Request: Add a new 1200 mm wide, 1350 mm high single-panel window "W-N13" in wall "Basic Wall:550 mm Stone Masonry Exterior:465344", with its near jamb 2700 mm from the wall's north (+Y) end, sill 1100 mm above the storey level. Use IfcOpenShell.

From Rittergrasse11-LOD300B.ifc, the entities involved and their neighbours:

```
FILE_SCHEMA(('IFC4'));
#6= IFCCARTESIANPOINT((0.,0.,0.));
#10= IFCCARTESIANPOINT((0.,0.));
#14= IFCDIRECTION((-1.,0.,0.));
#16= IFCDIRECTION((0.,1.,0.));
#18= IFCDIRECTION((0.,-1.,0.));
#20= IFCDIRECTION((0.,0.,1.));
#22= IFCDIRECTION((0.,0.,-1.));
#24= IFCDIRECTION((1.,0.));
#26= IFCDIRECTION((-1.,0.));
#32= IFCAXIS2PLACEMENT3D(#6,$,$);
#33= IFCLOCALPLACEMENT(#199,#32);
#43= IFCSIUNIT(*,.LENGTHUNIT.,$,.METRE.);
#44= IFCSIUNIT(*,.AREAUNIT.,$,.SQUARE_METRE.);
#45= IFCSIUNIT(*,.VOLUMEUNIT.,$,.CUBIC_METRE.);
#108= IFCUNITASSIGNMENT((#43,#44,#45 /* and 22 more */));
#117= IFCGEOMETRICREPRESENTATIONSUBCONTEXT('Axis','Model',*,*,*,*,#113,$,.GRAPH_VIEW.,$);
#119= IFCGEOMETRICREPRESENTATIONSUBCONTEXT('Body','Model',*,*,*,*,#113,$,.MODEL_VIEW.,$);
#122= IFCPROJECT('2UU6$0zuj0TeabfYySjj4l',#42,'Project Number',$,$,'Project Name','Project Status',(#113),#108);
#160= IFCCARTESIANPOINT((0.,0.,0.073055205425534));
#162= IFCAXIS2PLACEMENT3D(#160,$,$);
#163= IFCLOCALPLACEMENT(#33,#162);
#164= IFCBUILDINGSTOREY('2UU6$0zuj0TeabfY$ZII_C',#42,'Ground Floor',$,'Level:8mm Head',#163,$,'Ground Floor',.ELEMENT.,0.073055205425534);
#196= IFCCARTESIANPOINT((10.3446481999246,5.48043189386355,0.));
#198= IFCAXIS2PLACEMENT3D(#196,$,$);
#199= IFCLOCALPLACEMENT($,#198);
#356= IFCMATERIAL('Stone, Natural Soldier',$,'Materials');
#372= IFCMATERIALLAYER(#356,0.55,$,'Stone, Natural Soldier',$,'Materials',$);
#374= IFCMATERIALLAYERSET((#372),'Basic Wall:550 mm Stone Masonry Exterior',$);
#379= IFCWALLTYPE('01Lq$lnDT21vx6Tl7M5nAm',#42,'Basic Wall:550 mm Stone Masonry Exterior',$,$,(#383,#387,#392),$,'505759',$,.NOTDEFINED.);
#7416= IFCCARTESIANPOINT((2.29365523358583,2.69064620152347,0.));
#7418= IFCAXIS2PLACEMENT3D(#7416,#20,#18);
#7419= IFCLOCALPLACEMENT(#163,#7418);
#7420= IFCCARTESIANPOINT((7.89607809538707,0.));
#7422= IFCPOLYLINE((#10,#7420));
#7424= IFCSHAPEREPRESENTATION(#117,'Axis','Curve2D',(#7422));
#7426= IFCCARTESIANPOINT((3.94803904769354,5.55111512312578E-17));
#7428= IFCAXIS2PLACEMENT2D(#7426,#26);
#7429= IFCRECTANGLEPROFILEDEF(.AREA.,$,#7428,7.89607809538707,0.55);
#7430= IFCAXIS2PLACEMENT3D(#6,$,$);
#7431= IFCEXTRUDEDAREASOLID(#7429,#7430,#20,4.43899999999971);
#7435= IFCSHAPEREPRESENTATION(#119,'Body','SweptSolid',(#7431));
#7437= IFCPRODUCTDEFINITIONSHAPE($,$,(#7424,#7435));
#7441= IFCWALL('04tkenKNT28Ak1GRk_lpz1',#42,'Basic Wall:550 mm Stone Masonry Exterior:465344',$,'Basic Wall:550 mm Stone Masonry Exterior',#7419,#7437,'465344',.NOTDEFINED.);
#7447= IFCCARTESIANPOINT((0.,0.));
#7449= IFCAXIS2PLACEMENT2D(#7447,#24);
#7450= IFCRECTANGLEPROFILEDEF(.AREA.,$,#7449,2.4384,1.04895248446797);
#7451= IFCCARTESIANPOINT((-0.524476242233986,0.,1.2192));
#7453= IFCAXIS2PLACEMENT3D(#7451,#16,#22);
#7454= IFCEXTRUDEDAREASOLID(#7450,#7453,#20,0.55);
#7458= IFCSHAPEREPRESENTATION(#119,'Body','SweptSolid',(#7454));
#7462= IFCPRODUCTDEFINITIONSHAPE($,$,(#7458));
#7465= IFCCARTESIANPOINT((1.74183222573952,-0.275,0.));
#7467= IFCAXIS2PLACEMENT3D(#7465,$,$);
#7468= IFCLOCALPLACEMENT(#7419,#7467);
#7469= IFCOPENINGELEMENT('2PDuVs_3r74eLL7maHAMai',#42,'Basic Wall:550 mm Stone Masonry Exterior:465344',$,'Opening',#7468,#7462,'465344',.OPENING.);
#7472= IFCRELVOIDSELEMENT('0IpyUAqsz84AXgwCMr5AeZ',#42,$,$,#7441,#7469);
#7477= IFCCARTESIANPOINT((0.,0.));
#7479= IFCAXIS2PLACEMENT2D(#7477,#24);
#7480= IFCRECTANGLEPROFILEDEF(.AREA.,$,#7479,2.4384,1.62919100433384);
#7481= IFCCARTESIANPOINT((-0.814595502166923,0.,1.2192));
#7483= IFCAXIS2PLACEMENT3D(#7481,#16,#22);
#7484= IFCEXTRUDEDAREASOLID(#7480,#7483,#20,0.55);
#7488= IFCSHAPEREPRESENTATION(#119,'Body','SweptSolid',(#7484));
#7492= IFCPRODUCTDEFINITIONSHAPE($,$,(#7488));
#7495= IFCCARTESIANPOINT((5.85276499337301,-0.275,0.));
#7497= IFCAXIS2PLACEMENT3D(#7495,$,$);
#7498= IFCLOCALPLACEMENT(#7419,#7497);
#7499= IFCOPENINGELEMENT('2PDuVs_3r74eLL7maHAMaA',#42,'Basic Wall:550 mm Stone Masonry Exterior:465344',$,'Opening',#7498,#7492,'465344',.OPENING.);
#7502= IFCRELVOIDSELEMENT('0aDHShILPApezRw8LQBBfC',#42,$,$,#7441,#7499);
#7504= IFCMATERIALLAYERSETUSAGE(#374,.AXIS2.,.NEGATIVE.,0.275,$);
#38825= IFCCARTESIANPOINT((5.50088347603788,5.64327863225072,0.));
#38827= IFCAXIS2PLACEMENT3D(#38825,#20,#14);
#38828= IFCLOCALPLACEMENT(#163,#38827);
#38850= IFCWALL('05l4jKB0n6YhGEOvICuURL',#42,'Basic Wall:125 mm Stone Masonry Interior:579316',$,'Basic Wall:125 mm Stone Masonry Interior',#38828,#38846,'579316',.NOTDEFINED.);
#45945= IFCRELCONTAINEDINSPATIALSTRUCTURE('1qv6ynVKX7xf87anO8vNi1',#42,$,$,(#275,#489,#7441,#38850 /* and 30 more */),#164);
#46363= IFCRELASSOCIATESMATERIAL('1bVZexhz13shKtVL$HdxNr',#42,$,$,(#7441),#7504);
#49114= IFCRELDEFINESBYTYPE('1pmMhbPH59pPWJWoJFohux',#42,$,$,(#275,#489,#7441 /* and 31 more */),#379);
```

```python
import numpy as np
import ifcopenshell
import ifcopenshell.api.feature
import ifcopenshell.api.geometry
import ifcopenshell.api.root
import ifcopenshell.api.spatial
import ifcopenshell.geom
import ifcopenshell.util.element
import ifcopenshell.util.placement
import ifcopenshell.util.representation
import ifcopenshell.util.shape
import ifcopenshell.util.unit

model = ifcopenshell.open("Rittergrasse11-LOD300B.ifc")
unit_scale = ifcopenshell.util.unit.calculate_unit_scale(model)
settings = ifcopenshell.geom.settings()


def volume(element):
    """Net volume in cubic metres, openings subtracted."""
    shape = ifcopenshell.geom.create_shape(settings, element)
    return ifcopenshell.util.shape.get_volume(shape.geometry)


wall = model.by_guid("04tkenKNT28Ak1GRk_lpz1")
storey = ifcopenshell.util.element.get_container(wall, ifc_class="IfcBuildingStorey")
context = ifcopenshell.util.representation.get_context(model, "Model", "Body", "MODEL_VIEW")
before = volume(wall)

width, height, from_end, sill = 1.2, 1.35, 2.7, 1.1  # metres

# The wall runs along its own X axis, and the end named is its -X end.
wall_shape = ifcopenshell.geom.create_shape(settings, wall)
x, y, z = ifcopenshell.util.shape.get_vertices(wall_shape.geometry).T
start = x.min() + from_end
face, thickness = float(y.min()), float(y.max() - y.min())
wall_matrix = ifcopenshell.util.placement.get_local_placement(wall.ObjectPlacement)
level = ifcopenshell.util.placement.get_local_placement(storey.ObjectPlacement)[2, 3]


def in_wall(x, y):
    """Placement at x, y metres in the wall's axes, at sill height."""
    matrix = wall_matrix.copy()
    matrix[:, 3] = wall_matrix @ np.array([x / unit_scale, y / unit_scale, 0.0, 1.0])
    matrix[2, 3] = level + sill / unit_scale
    return matrix


# Opening: a box that overshoots both wall faces by 50 mm.
opening = ifcopenshell.api.root.create_entity(model, ifc_class="IfcOpeningElement", predefined_type="OPENING")
box = ifcopenshell.api.geometry.add_wall_representation(
    model, context=context, length=width, height=height, thickness=thickness + 0.1
)
ifcopenshell.api.geometry.assign_representation(model, product=opening, representation=box)
ifcopenshell.api.geometry.edit_object_placement(model, product=opening, matrix=in_wall(start, face - 0.05), is_si=False)
ifcopenshell.api.feature.add_feature(model, feature=opening, element=wall)

window = ifcopenshell.api.root.create_entity(model, ifc_class="IfcWindow", name="W-N13", predefined_type="WINDOW")
window.OverallWidth, window.OverallHeight = width / unit_scale, height / unit_scale
window.PartitioningType = "SINGLE_PANEL"
body = ifcopenshell.api.geometry.add_window_representation(
    model,
    context=context,
    overall_width=window.OverallWidth,
    overall_height=window.OverallHeight,
    partition_type="SINGLE_PANEL",
)
ifcopenshell.api.geometry.assign_representation(model, product=window, representation=body)
ifcopenshell.api.spatial.assign_container(model, products=[window], relating_structure=storey)
ifcopenshell.api.feature.add_filling(model, opening=opening, element=window)

# Centre the window in the wall's thickness.
ifcopenshell.api.geometry.edit_object_placement(model, product=window, matrix=in_wall(start, face), is_si=False)
window_shape = ifcopenshell.geom.create_shape(settings, window)
depth = ifcopenshell.util.shape.get_vertices(window_shape.geometry)[:, 1]
offset = face + thickness / 2 - (depth.min() + depth.max()) / 2
ifcopenshell.api.geometry.edit_object_placement(model, product=window, matrix=in_wall(start, offset), is_si=False)

after = volume(wall)

print(f"wall volume {before:.3f} -> {after:.3f} m3")

model.write("Rittergrasse11-LOD300B_updated.ifc")
```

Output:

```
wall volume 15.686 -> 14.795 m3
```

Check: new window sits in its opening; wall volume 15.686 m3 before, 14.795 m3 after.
